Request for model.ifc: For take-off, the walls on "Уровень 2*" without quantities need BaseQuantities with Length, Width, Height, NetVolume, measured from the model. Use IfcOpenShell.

First a look at what the model holds.

```python
import ifcopenshell
import ifcopenshell.util.element
import ifcopenshell.util.unit

model = ifcopenshell.open("model.ifc")
print(model.schema)
for unit_type in ("LENGTHUNIT", "AREAUNIT", "VOLUMEUNIT"):
    print(unit_type, ifcopenshell.util.unit.calculate_unit_scale(model, unit_type))
storey = next(s for s in model.by_type("IfcBuildingStorey") if s.Name == "Уровень 2*")
walls = [e for e in ifcopenshell.util.element.get_decomposition(storey) if e.is_a("IfcWall")]
for e in sorted(walls, key=lambda e: e.id()):
    print(e.id(), e.is_a(), e.Name, list(ifcopenshell.util.element.get_psets(e, qtos_only=True)), sep=" | ")
```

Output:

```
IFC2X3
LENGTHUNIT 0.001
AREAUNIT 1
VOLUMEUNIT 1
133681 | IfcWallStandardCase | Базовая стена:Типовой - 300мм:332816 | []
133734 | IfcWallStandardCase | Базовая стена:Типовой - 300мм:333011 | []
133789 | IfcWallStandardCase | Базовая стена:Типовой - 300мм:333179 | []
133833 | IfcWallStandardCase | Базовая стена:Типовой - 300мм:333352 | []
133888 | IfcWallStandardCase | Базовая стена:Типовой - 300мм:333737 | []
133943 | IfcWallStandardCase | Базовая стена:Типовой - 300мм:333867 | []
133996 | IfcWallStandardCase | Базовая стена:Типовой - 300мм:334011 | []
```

```python
import ifcopenshell
import ifcopenshell.api.pset
import ifcopenshell.geom
import ifcopenshell.util.element
import ifcopenshell.util.shape
import ifcopenshell.util.unit

model = ifcopenshell.open("model.ifc")
unit_scale = ifcopenshell.util.unit.calculate_unit_scale(model)
volume_scale = ifcopenshell.util.unit.calculate_unit_scale(model, "VOLUMEUNIT")
settings = ifcopenshell.geom.settings()

storey = next(s for s in model.by_type("IfcBuildingStorey") if s.Name == "Уровень 2*")
walls = [e for e in ifcopenshell.util.element.get_decomposition(storey) if e.is_a("IfcWall")]

for e in sorted(walls, key=lambda e: e.id()):
    if ifcopenshell.util.element.get_psets(e, qtos_only=True, should_inherit=False):
        continue
    # Geometry comes back in metres, in the element's own axes.
    shape = ifcopenshell.geom.create_shape(settings, e)
    values = {
        "Length": ifcopenshell.util.shape.get_x(shape.geometry) / unit_scale,
        "Width": ifcopenshell.util.shape.get_y(shape.geometry) / unit_scale,
        "Height": ifcopenshell.util.shape.get_z(shape.geometry) / unit_scale,
        "NetVolume": ifcopenshell.util.shape.get_volume(shape.geometry) / volume_scale,
    }
    qto = ifcopenshell.api.pset.add_qto(model, product=e, name="BaseQuantities")
    ifcopenshell.api.pset.edit_qto(model, qto=qto, properties=values)
    print(e.id(), {k: round(v, 3) for k, v in values.items()})

model.write("model_v2.ifc")
```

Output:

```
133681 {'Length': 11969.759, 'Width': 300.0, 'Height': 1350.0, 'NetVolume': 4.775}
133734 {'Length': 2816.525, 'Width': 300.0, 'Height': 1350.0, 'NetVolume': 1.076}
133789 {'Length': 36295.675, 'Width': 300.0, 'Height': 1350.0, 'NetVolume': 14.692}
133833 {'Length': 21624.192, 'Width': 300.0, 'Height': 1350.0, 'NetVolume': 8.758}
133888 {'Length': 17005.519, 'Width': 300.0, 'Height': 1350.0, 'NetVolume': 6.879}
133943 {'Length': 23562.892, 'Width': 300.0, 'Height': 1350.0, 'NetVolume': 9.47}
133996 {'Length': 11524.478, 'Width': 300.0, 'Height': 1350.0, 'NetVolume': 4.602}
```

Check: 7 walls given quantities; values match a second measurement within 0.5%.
